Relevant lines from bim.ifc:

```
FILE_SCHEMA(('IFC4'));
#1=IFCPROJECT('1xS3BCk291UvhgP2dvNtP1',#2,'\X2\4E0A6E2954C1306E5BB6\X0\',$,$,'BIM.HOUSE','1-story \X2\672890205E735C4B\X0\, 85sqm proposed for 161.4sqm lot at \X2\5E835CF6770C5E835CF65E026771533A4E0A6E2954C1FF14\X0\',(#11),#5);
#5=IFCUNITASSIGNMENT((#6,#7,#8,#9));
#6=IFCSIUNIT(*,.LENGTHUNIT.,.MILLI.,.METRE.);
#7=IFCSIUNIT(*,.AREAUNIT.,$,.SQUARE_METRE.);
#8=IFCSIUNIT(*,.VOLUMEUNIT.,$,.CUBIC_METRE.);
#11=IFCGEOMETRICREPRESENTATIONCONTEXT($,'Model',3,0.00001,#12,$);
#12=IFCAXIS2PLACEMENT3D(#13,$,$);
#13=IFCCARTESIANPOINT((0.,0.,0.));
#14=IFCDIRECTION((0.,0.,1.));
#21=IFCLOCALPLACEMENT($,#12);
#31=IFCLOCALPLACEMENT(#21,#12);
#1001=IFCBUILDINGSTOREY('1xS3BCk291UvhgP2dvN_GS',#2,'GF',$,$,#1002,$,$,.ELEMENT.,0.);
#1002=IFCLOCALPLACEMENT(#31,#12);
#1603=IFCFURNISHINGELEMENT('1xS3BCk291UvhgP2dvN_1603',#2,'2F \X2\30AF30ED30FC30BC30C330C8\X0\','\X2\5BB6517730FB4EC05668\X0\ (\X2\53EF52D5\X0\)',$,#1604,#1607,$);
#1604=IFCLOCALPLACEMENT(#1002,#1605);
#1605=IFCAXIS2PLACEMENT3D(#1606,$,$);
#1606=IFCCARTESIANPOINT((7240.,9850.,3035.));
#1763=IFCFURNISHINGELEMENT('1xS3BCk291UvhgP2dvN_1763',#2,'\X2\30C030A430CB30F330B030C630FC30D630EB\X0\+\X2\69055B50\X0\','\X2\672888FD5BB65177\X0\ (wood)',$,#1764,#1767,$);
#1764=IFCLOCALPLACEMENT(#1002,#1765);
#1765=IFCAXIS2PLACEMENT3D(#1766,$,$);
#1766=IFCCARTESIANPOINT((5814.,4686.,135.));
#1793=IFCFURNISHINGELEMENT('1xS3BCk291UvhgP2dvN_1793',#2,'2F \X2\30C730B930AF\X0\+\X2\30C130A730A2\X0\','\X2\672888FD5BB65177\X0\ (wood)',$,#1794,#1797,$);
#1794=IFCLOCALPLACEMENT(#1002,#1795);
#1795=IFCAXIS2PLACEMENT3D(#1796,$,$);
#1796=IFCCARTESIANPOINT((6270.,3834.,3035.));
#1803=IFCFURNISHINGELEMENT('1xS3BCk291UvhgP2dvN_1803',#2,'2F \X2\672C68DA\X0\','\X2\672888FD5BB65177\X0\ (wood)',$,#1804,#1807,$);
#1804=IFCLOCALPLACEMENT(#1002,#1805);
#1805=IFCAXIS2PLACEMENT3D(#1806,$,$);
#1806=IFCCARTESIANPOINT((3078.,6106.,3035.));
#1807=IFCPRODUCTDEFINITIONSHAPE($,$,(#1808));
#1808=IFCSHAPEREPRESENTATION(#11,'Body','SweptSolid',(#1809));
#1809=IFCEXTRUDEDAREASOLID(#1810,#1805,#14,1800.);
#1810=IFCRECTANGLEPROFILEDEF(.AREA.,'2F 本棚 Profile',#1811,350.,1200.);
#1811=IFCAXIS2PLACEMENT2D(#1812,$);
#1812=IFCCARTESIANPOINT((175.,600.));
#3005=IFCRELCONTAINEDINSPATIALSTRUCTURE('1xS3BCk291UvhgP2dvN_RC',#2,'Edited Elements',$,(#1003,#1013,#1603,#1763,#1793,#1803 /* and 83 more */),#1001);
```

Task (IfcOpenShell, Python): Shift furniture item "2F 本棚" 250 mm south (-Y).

```python
import ifcopenshell
import ifcopenshell.api.geometry
import ifcopenshell.util.placement

model = ifcopenshell.open("bim.ifc")

item = model.by_id(1803)
matrix = ifcopenshell.util.placement.get_local_placement(item.ObjectPlacement)
matrix[1, 3] -= 250.0
ifcopenshell.api.geometry.edit_object_placement(model, product=item, matrix=matrix, is_si=False)

print(ifcopenshell.util.placement.get_local_placement(item.ObjectPlacement).round(3) + 0.0)

model.write("bim_rev.ifc")
```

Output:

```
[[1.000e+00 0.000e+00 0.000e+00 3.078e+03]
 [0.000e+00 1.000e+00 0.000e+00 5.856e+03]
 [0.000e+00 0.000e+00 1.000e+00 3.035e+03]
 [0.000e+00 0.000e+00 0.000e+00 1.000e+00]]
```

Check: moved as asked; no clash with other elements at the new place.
